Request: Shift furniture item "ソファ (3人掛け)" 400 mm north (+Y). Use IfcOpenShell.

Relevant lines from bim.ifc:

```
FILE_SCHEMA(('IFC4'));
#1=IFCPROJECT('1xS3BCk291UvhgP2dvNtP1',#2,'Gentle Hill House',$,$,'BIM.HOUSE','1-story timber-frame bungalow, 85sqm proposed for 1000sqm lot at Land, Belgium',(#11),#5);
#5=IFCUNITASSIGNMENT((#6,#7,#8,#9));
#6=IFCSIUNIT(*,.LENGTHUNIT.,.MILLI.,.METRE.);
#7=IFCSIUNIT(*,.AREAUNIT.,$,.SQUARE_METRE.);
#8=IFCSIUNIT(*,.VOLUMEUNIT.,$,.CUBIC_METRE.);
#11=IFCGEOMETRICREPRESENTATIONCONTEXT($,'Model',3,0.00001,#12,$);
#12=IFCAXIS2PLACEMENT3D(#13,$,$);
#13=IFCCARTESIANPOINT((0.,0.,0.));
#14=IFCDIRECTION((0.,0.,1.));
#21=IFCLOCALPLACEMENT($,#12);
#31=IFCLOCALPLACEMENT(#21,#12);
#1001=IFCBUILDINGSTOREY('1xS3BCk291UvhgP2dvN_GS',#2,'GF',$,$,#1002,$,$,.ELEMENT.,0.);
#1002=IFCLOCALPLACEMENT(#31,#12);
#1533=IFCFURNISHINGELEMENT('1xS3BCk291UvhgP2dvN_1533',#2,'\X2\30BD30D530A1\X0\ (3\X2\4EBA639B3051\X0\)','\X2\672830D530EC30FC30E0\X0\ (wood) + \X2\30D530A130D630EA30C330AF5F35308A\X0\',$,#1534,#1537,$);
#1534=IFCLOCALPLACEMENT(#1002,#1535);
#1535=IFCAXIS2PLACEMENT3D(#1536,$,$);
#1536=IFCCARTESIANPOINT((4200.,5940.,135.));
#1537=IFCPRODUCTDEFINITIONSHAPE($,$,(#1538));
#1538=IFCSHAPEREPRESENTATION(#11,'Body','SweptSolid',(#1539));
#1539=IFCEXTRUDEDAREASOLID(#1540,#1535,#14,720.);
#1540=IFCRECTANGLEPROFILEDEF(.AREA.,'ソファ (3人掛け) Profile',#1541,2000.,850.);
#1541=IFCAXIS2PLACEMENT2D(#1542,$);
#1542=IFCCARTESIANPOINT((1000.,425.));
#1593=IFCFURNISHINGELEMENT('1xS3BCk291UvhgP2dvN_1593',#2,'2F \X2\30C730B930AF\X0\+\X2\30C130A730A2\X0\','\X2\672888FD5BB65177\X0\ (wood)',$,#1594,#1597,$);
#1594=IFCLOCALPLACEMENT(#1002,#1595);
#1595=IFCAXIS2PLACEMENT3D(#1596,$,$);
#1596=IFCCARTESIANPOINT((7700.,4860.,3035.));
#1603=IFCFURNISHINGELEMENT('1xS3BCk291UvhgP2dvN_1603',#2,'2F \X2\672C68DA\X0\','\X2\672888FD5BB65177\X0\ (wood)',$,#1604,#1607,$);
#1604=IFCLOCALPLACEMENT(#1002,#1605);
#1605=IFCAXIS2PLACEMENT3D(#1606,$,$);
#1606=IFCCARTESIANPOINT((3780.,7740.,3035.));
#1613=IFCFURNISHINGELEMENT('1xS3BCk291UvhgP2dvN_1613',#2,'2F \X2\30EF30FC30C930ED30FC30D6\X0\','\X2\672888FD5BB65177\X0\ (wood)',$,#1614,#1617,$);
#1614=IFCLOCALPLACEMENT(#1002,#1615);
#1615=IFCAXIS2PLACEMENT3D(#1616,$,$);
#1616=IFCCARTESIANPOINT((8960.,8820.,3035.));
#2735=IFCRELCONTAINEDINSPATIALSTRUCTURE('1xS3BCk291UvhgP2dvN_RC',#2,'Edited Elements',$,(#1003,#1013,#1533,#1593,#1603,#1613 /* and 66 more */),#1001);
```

```python
import ifcopenshell
import ifcopenshell.api.geometry
import ifcopenshell.util.placement
import ifcopenshell.util.unit

model = ifcopenshell.open("bim.ifc")
unit_scale = ifcopenshell.util.unit.calculate_unit_scale(model)

item = model.by_guid("1xS3BCk291UvhgP2dvN_1533")
matrix = ifcopenshell.util.placement.get_local_placement(item.ObjectPlacement)
matrix[1, 3] += 0.4 / unit_scale
ifcopenshell.api.geometry.edit_object_placement(model, product=item, matrix=matrix, is_si=False)

print(ifcopenshell.util.placement.get_local_placement(item.ObjectPlacement).round(3) + 0.0)

model.write("bim-out.ifc")
```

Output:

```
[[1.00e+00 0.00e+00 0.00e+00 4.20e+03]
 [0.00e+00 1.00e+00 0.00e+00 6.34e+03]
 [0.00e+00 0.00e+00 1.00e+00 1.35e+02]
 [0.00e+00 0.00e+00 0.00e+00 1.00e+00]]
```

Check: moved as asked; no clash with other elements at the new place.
